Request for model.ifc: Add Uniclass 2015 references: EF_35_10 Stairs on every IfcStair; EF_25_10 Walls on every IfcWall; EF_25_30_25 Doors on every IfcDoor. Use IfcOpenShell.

First a look at what the model holds.

```python
import ifcopenshell

model = ifcopenshell.open("model.ifc")
print(model.schema)
print("classifications:", [c.Name for c in model.by_type("IfcClassification")])
for ifc_class in ("IfcDoor", "IfcRoof", "IfcStair", "IfcWall", "IfcWindow"):
    print(ifc_class, len(model.by_type(ifc_class)))
```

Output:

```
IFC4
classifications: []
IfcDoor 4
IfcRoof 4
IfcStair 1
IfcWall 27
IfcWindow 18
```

```python
import ifcopenshell
import ifcopenshell.api.classification

model = ifcopenshell.open("model.ifc")

system = ifcopenshell.api.classification.add_classification(model, classification="Uniclass 2015")

codes = {
    "IfcStair": ("EF_35_10", "Stairs"),
    "IfcWall": ("EF_25_10", "Walls"),
    "IfcDoor": ("EF_25_30_25", "Doors"),
}
for ifc_class, (code, name) in codes.items():
    products = model.by_type(ifc_class)
    ifcopenshell.api.classification.add_reference(
        model, products=products, classification=system, identification=code, name=name
    )
    print(code, len(products))

model.write("model_updated.ifc")
```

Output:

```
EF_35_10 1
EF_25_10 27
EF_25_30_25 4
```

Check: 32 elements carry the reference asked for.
